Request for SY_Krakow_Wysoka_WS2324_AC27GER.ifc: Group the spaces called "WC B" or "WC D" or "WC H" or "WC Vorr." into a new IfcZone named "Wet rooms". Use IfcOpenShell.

First a look at what the model holds.

```python
import ifcopenshell

model = ifcopenshell.open("SY_Krakow_Wysoka_WS2324_AC27GER.ifc")
print(model.schema)
seen = {}
for space in model.by_type("IfcSpace"):
    seen[space.LongName] = seen.get(space.LongName, 0) + 1
for name, count in sorted(seen.items(), key=str):
    print(count, "x", name)
print("zones:", [z.Name for z in model.by_type("IfcZone")][:20])
```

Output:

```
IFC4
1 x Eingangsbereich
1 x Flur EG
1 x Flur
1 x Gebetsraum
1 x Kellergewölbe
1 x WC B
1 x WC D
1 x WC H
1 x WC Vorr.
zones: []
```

```python
import ifcopenshell
import ifcopenshell.api.group
import ifcopenshell.api.root

model = ifcopenshell.open("SY_Krakow_Wysoka_WS2324_AC27GER.ifc")

names = {"WC B", "WC D", "WC H", "WC Vorr."}
spaces = [s for s in model.by_type("IfcSpace") if s.LongName in names]

zone = ifcopenshell.api.root.create_entity(model, ifc_class="IfcZone", name="Wet rooms")
ifcopenshell.api.group.assign_group(model, products=spaces, group=zone)
print(len(spaces), "spaces in", zone.Name)

model.write("SY_Krakow_Wysoka_WS2324_AC27GER_rev.ifc")
```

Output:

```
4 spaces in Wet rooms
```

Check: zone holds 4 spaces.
